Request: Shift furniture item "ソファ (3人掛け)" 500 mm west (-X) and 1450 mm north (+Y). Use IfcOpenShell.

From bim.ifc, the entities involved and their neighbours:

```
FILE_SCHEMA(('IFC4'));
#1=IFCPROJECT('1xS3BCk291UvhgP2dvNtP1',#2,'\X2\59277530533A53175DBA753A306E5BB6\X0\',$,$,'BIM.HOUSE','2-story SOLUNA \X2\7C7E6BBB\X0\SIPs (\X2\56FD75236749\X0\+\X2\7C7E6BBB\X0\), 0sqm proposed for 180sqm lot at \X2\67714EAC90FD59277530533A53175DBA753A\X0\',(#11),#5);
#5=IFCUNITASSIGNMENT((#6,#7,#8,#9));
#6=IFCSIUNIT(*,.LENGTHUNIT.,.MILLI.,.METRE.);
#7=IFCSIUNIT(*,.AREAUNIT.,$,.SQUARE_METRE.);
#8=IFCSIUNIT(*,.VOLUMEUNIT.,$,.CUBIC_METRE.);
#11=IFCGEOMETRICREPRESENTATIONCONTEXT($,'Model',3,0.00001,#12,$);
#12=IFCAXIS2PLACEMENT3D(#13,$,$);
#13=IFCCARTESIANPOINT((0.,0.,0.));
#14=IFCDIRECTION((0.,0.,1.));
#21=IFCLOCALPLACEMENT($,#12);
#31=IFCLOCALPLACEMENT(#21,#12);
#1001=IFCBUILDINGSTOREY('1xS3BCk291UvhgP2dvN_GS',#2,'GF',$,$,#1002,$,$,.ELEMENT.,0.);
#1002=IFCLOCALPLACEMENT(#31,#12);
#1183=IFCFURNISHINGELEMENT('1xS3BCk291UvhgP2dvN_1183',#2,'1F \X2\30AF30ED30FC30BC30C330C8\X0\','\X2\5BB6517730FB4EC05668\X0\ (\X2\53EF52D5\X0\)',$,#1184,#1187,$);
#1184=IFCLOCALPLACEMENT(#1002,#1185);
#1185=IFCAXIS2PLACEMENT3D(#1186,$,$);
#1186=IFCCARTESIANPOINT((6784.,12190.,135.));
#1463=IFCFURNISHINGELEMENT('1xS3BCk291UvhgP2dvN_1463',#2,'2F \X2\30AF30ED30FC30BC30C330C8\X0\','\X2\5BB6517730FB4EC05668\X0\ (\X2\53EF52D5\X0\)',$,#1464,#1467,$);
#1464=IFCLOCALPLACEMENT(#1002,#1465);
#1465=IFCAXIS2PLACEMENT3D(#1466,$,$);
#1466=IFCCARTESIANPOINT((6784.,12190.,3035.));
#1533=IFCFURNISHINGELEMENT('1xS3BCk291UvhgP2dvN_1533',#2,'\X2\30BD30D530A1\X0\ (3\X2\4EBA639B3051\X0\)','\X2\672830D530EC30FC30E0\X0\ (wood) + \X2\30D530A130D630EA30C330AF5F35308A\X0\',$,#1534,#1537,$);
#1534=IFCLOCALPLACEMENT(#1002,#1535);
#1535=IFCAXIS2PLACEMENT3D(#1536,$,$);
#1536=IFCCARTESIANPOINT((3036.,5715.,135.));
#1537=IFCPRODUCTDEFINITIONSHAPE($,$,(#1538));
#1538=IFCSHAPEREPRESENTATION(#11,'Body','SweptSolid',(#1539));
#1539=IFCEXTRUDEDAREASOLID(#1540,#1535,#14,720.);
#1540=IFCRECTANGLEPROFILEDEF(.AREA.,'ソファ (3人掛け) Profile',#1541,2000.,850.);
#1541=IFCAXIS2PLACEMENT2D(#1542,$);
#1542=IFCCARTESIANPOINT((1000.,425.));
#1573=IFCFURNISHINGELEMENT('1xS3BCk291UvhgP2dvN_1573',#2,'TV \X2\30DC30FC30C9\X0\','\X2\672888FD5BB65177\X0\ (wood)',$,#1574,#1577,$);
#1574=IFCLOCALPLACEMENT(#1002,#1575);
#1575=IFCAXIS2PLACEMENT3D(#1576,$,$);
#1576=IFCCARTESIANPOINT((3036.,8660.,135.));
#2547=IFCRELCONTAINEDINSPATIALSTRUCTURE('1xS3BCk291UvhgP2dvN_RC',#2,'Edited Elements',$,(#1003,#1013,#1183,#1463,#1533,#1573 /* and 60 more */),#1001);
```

```python
import ifcopenshell
import ifcopenshell.api.geometry
import ifcopenshell.util.placement
import ifcopenshell.util.unit

model = ifcopenshell.open("bim.ifc")
unit_scale = ifcopenshell.util.unit.calculate_unit_scale(model)

item = model.by_guid("1xS3BCk291UvhgP2dvN_1533")
matrix = ifcopenshell.util.placement.get_local_placement(item.ObjectPlacement)
matrix[0, 3] -= 0.5 / unit_scale
matrix[1, 3] += 1.45 / unit_scale
ifcopenshell.api.geometry.edit_object_placement(model, product=item, matrix=matrix, is_si=False)

print(ifcopenshell.util.placement.get_local_placement(item.ObjectPlacement).round(3) + 0.0)

model.write("bim_updated.ifc")
```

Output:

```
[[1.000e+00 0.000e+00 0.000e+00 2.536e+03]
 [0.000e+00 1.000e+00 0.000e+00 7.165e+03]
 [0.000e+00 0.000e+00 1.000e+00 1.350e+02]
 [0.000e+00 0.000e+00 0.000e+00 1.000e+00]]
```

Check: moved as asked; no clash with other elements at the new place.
